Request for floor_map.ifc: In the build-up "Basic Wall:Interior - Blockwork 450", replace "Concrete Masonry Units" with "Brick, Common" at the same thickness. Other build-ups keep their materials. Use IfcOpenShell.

First a look at what the model holds.

```python
import ifcopenshell
import ifcopenshell.util.element

model = ifcopenshell.open("floor_map.ifc")
print(model.schema)
for layer_set in model.by_type("IfcMaterialLayerSet"):
    if layer_set.LayerSetName == "Basic Wall:Interior - Blockwork 450":
        for layer in layer_set.MaterialLayers:
            print(layer.id(), layer.Material and layer.Material.Name, layer.LayerThickness, sep=" | ")
        print(len(ifcopenshell.util.element.get_elements_by_material(model, layer_set)), "elements and types use it")
print(sorted(m.Name for m in model.by_type("IfcMaterial") if m.Name)[:60])
```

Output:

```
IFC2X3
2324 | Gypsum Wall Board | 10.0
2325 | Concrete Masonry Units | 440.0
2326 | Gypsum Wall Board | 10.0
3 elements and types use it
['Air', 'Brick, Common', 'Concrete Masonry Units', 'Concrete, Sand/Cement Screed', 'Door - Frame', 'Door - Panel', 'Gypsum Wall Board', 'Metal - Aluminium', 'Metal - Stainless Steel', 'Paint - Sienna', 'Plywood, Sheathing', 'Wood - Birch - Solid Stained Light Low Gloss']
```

```python
import ifcopenshell
import ifcopenshell.api.material

model = ifcopenshell.open("floor_map.ifc")

layer_set = next(s for s in model.by_type("IfcMaterialLayerSet") if s.LayerSetName == "Basic Wall:Interior - Blockwork 450")
layer = next(l for l in layer_set.MaterialLayers if l.Material and l.Material.Name == "Concrete Masonry Units")
material = next(m for m in model.by_type("IfcMaterial") if m.Name == "Brick, Common")

# Point this one layer at the other material; renaming the old one would change it everywhere.
ifcopenshell.api.material.edit_layer(model, layer=layer, attributes={}, material=material)

print([l.Material.Name if l.Material else None for l in layer_set.MaterialLayers])

model.write("floor_map-out.ifc")
```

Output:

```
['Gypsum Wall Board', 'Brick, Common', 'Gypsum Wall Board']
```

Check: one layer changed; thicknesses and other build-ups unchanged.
